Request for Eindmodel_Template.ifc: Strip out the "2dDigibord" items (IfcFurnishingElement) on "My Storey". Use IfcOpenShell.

First a look at what the model holds.

```python
import ifcopenshell
import ifcopenshell.util.element

model = ifcopenshell.open("Eindmodel_Template.ifc")
print(model.schema)
storey = next(s for s in model.by_type("IfcBuildingStorey") if s.Name == "My Storey")
furniture = [e for e in ifcopenshell.util.element.get_decomposition(storey) if e.is_a("IfcFurnishingElement")]
seen = {}
for e in furniture:
    element_type = ifcopenshell.util.element.get_type(e)
    name = element_type.Name if element_type not in (None, e) else None
    seen[name] = seen.get(name, 0) + 1
for name, count in sorted(seen.items(), key=str):
    print(count, "x", name)
```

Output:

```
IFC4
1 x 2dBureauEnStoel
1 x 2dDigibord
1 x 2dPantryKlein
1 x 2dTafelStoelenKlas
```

```python
import ifcopenshell
import ifcopenshell.api.root
import ifcopenshell.util.element

model = ifcopenshell.open("Eindmodel_Template.ifc")

storey = next(s for s in model.by_type("IfcBuildingStorey") if s.Name == "My Storey")
furniture = [e for e in ifcopenshell.util.element.get_decomposition(storey) if e.is_a("IfcFurnishingElement")]
targets = [e for e in furniture if (t := ifcopenshell.util.element.get_type(e)) not in (None, e) and t.Name == "2dDigibord"]

for e in targets:
    ifcopenshell.api.root.remove_product(model, product=e)
print(len(targets), "removed")

model.write("Eindmodel_Template-out.ifc")
```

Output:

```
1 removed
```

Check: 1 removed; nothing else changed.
